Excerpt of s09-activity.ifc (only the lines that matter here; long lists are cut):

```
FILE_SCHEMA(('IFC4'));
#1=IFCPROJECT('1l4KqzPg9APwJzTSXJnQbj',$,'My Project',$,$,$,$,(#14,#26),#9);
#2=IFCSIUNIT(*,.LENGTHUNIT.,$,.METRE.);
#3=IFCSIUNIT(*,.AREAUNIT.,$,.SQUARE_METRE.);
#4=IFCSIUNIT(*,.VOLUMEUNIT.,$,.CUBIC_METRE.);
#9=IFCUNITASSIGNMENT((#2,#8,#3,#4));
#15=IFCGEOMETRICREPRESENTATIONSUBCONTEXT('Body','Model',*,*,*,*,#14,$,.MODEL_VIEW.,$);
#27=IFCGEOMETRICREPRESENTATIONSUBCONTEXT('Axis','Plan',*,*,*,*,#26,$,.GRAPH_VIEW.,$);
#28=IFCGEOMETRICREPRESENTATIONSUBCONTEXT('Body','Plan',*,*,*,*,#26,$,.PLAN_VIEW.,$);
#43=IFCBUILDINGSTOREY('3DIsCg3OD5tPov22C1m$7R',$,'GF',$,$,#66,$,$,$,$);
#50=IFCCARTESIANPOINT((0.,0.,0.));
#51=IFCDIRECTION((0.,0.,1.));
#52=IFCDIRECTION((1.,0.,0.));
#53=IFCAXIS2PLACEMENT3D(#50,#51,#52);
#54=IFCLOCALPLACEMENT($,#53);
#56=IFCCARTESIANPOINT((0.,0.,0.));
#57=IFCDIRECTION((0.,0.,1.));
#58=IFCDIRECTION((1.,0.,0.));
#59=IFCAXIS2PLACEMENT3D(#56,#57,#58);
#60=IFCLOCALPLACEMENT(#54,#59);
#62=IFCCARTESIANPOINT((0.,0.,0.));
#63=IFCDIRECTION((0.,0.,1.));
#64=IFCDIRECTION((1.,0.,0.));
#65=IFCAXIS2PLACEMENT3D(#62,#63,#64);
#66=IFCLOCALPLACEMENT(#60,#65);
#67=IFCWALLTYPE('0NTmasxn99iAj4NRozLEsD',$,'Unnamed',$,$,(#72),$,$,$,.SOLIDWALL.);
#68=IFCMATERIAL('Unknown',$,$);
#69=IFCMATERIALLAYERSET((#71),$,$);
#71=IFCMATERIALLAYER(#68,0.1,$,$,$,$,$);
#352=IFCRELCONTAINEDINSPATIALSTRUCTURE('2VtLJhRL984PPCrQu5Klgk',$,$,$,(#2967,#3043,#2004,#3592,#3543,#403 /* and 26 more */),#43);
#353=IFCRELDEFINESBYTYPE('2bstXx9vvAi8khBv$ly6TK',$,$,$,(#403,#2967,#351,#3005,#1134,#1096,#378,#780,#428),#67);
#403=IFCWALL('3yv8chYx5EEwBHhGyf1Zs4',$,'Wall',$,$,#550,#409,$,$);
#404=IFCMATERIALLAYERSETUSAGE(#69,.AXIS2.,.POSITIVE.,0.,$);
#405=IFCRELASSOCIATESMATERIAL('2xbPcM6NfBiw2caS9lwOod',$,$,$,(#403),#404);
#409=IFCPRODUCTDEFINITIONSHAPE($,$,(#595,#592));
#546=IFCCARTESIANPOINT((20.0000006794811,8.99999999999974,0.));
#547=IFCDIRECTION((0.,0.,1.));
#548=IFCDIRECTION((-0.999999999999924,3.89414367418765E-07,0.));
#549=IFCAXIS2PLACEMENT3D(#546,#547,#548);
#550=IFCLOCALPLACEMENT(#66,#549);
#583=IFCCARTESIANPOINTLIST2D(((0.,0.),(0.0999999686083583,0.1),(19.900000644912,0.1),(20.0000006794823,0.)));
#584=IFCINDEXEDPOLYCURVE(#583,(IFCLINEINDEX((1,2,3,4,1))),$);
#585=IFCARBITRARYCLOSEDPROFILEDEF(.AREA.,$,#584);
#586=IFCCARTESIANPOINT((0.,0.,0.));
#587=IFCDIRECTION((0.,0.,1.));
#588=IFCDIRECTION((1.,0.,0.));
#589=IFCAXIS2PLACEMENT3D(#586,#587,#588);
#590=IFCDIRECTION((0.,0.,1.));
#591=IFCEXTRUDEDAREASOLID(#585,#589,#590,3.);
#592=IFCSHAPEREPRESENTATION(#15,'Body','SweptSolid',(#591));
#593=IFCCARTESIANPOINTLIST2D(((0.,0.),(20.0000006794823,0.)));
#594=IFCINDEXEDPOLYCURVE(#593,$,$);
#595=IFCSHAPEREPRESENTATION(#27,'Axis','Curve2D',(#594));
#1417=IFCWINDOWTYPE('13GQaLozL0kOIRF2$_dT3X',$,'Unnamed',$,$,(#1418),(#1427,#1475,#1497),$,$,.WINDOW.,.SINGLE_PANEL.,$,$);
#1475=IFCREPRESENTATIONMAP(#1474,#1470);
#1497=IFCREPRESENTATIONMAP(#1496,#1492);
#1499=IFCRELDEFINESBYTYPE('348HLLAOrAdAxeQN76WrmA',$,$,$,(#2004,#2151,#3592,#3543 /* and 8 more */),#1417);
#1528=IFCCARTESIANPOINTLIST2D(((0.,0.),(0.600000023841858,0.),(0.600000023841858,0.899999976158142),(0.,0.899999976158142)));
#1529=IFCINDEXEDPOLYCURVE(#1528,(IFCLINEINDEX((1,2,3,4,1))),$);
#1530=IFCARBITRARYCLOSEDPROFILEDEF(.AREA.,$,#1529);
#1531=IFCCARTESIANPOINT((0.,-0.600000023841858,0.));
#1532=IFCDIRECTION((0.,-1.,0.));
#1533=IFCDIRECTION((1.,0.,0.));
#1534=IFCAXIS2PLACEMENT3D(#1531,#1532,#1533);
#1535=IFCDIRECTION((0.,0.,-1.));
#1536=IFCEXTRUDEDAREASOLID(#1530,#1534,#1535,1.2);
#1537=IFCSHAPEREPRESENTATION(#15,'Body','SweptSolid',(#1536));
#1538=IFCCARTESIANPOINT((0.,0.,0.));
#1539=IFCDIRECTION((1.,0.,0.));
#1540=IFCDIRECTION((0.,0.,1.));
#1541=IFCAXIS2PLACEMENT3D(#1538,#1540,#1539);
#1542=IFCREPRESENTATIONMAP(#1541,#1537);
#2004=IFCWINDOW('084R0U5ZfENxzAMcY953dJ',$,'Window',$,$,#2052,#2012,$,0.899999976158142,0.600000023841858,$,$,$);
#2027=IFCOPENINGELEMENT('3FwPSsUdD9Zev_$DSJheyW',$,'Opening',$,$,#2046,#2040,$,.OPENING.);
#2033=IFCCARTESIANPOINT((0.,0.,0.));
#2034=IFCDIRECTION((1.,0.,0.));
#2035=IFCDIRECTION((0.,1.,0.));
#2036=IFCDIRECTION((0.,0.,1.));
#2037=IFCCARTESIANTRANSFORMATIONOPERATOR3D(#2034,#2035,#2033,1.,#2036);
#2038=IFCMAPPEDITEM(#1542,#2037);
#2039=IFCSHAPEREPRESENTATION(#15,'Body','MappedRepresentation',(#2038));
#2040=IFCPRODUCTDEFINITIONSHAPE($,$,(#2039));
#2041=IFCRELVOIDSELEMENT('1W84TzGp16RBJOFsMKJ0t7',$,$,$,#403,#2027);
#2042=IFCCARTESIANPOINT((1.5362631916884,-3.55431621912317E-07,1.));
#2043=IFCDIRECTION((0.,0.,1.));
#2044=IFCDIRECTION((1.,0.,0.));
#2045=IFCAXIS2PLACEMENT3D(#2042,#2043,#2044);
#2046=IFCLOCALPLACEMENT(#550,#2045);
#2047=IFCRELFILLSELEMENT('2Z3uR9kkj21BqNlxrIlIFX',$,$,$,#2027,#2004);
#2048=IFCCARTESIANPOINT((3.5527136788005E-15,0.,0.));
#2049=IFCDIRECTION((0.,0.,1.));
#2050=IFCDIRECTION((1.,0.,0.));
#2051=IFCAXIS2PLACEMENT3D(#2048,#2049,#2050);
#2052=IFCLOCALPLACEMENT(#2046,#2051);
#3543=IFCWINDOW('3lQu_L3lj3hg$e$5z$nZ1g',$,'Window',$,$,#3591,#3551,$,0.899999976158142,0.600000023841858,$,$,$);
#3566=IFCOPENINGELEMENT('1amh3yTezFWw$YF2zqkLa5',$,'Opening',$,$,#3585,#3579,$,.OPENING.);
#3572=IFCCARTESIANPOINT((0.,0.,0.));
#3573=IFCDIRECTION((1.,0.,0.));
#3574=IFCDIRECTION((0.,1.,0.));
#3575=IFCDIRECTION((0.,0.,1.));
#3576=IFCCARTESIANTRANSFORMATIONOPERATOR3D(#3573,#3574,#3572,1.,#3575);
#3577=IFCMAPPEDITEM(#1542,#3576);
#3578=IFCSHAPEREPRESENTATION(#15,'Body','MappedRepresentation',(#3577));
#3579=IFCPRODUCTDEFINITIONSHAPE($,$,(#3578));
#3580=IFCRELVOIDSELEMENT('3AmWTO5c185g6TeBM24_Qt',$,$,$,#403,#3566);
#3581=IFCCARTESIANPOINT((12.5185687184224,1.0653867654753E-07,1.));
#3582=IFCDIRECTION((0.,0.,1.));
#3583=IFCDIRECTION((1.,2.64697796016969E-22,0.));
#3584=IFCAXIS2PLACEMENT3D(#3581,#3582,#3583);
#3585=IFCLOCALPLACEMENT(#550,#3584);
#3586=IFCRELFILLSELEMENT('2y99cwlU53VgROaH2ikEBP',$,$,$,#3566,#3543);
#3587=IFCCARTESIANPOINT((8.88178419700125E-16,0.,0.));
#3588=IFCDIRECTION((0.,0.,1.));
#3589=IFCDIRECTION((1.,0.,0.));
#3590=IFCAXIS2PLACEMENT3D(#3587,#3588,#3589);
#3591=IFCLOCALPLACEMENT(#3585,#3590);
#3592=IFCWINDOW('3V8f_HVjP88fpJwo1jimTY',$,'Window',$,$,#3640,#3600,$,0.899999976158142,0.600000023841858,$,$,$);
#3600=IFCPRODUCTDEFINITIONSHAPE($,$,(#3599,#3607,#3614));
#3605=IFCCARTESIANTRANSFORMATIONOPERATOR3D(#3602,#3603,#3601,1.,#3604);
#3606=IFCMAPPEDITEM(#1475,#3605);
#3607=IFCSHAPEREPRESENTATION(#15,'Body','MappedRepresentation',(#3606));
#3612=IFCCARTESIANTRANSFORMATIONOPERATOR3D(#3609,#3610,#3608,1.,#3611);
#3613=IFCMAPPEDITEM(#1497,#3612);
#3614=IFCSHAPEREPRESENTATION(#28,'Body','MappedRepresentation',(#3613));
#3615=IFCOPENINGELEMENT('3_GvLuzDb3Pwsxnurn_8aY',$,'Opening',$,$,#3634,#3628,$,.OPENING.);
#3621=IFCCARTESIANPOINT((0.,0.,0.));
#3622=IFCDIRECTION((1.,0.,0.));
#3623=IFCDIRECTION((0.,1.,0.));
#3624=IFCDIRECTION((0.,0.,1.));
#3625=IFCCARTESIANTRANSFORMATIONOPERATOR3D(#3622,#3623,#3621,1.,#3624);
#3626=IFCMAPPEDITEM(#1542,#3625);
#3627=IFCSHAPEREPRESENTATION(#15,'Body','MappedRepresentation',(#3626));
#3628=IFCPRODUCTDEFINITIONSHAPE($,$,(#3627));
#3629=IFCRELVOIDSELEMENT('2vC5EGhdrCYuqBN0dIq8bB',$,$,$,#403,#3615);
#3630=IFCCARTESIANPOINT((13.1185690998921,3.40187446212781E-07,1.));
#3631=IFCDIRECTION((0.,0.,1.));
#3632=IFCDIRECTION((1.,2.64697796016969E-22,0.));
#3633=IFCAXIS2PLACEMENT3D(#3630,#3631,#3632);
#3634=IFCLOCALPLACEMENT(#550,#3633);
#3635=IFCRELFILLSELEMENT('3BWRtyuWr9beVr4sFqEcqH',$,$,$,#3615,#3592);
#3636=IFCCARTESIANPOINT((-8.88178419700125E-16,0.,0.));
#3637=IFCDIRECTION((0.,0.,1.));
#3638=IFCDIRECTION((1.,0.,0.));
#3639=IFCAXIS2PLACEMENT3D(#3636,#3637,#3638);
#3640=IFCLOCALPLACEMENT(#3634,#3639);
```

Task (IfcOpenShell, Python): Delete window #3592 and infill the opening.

```python
import ifcopenshell
import ifcopenshell.api.feature
import ifcopenshell.api.root
import ifcopenshell.geom
import ifcopenshell.util.shape

model = ifcopenshell.open("s09-activity.ifc")
settings = ifcopenshell.geom.settings()


def volume(element):
    """Net volume in cubic metres, openings subtracted."""
    shape = ifcopenshell.geom.create_shape(settings, element)
    return ifcopenshell.util.shape.get_volume(shape.geometry)


window = model.by_guid("3V8f_HVjP88fpJwo1jimTY")
opening = window.FillsVoids[0].RelatingOpeningElement
wall = opening.VoidsElements[0].RelatingBuildingElement
before = volume(wall)

ifcopenshell.api.root.remove_product(model, product=window)
ifcopenshell.api.feature.remove_feature(model, feature=opening)

after = volume(wall)

print(f"wall volume {before:.3f} -> {after:.3f} m3")

model.write("s09-activity_updated.ifc")
```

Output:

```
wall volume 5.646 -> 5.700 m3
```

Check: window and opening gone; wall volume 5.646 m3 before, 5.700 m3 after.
